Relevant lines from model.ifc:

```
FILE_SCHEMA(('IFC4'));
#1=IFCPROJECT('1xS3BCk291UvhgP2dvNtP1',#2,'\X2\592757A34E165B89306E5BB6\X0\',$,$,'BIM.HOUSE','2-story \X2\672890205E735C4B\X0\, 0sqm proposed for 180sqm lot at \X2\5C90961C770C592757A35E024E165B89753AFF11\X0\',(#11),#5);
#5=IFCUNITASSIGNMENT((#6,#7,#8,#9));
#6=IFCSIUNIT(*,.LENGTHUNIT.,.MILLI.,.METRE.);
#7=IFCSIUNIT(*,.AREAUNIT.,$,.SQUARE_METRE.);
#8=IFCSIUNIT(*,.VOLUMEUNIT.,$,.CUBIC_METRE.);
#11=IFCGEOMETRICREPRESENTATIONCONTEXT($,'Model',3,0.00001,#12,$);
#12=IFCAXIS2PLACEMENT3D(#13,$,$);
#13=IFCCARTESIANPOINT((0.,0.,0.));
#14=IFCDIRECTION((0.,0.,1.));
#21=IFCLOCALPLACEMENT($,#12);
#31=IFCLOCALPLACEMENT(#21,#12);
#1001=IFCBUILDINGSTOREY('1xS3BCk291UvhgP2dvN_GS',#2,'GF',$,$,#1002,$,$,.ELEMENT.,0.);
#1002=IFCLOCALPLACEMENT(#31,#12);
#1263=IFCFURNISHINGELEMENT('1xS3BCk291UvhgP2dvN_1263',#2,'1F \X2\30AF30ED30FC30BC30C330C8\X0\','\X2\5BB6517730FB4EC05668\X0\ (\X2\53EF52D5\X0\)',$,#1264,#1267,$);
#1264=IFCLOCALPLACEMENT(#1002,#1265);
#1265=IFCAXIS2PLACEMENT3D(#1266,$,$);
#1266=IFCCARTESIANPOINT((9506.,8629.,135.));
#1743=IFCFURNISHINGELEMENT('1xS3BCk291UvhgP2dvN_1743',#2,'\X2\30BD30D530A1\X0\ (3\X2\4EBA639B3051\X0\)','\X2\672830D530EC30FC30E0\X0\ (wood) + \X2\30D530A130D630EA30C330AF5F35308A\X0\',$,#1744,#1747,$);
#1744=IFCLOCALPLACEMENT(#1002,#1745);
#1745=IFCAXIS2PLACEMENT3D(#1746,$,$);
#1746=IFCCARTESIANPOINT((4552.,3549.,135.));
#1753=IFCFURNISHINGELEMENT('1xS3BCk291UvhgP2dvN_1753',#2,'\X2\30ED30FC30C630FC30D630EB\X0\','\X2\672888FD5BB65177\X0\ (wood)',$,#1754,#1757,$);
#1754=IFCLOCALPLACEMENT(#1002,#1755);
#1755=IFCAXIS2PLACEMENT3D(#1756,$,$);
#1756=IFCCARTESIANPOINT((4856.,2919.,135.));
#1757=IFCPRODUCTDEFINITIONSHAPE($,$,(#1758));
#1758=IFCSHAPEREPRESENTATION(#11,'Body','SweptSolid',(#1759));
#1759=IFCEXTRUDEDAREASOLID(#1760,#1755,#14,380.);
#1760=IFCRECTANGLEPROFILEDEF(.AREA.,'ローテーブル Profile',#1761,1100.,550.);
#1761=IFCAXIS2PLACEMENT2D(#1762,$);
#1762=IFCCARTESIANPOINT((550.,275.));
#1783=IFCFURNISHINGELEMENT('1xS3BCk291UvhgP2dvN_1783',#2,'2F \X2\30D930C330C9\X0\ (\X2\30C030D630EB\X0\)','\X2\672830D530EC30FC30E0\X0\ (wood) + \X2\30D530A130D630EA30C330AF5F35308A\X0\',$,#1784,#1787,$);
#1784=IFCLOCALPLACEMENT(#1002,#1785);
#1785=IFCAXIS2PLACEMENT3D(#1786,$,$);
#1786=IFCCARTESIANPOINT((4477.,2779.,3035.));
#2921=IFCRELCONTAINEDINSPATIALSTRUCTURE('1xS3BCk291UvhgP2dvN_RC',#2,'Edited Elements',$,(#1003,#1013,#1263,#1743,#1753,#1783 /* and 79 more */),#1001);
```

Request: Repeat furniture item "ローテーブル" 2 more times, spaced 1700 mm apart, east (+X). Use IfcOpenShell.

```python
import numpy as np
import ifcopenshell
import ifcopenshell.api.geometry
import ifcopenshell.api.root
import ifcopenshell.util.element
import ifcopenshell.util.placement
import ifcopenshell.util.unit

model = ifcopenshell.open("model.ifc")
unit_scale = ifcopenshell.util.unit.calculate_unit_scale(model)


def reuse_history(source, copy):
    """copy_class also copies each property set's owner history, people and application; keep the originals."""
    for rel in copy.IsDefinedBy:
        if rel.is_a("IfcRelDefinesByProperties") and (history := rel.RelatingPropertyDefinition.OwnerHistory):
            rel.RelatingPropertyDefinition.OwnerHistory = source.OwnerHistory
            ifcopenshell.util.element.remove_deep2(model, history)


source = model.by_id(1753)
base = ifcopenshell.util.placement.get_local_placement(source.ObjectPlacement)
step = np.array([1.0, 0.0, 0.0]) * 1.7 / unit_scale

for i in range(1, 3):
    copy = ifcopenshell.api.root.copy_class(model, product=source)
    copy.Representation = ifcopenshell.util.element.copy_deep(
        model, source.Representation, exclude=["IfcGeometricRepresentationContext", "IfcRepresentationMap"]
    )
    reuse_history(source, copy)
    matrix = base.copy()
    matrix[:3, 3] += i * step
    print("added at", matrix[:3, 3].round(3) + 0.0)
    ifcopenshell.api.geometry.edit_object_placement(model, product=copy, matrix=matrix, is_si=False)

model.write("model_edited.ifc")
```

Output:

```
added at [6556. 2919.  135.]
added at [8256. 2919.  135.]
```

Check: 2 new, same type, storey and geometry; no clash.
